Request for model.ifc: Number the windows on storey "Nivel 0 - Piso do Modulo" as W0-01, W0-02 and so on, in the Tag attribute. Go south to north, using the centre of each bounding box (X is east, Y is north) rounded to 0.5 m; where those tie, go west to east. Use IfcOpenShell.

First a look at what the model holds.

```python
import ifcopenshell
import ifcopenshell.util.element
import ifcopenshell.util.placement

model = ifcopenshell.open("model.ifc")
print(model.schema)
storey = next(s for s in model.by_type("IfcBuildingStorey") if s.Name == "Nivel 0 - Piso do Modulo")
windows = [e for e in ifcopenshell.util.element.get_decomposition(storey) if e.is_a("IfcWindow")]
for e in sorted(windows, key=lambda e: e.id()):
    origin = ifcopenshell.util.placement.get_local_placement(e.ObjectPlacement)[:3, 3]
    print(e.id(), e.Tag, e.Name, origin.round(2) + 0.0, sep=" | ")
```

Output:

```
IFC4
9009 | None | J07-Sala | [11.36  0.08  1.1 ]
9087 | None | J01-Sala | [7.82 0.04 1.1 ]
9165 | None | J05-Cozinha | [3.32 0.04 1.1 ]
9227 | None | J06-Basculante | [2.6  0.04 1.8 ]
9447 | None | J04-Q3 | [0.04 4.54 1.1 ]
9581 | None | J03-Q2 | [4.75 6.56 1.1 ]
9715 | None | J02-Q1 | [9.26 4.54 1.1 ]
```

```python
import ifcopenshell
import ifcopenshell.geom
import ifcopenshell.util.element
import ifcopenshell.util.shape

model = ifcopenshell.open("model.ifc")
settings = ifcopenshell.geom.settings()
settings.set("use-world-coords", True)


def centre(element):
    shape = ifcopenshell.geom.create_shape(settings, element)
    return ifcopenshell.util.shape.get_bbox_centroid(shape.geometry)


storey = next(s for s in model.by_type("IfcBuildingStorey") if s.Name == "Nivel 0 - Piso do Modulo")
windows = [e for e in ifcopenshell.util.element.get_decomposition(storey) if e.is_a("IfcWindow")]

# Insertion points can sit at a corner or the storey origin, so sort by the geometry (in metres).
centres = {e: centre(e) for e in windows}
windows.sort(key=lambda e: (round(centres[e][1] / 0.5), centres[e][0]))

for i, e in enumerate(windows, start=1):
    number = f"W0-{i:02d}"
    e.Tag = number
    print(e.id(), number)

model.write("model_edited.ifc")
```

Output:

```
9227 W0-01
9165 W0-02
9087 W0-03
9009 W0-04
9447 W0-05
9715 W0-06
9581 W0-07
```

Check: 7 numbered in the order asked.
